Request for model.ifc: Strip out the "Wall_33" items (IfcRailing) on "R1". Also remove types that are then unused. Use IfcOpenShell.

First a look at what the model holds.

```python
import ifcopenshell
import ifcopenshell.util.element

model = ifcopenshell.open("model.ifc")
print(model.schema)
storey = next(s for s in model.by_type("IfcBuildingStorey") if s.Name == "R1")
railings = [e for e in ifcopenshell.util.element.get_decomposition(storey) if e.is_a("IfcRailing")]
seen = {}
for e in railings:
    element_type = ifcopenshell.util.element.get_type(e)
    name = element_type.Name if element_type not in (None, e) else None
    seen[name] = seen.get(name, 0) + 1
for name, count in sorted(seen.items(), key=str):
    print(count, "x", name)
```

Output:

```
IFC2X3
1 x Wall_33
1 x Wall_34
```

```python
import ifcopenshell
import ifcopenshell.api.root
import ifcopenshell.util.element

model = ifcopenshell.open("model.ifc")

storey = next(s for s in model.by_type("IfcBuildingStorey") if s.Name == "R1")
railings = [e for e in ifcopenshell.util.element.get_decomposition(storey) if e.is_a("IfcRailing")]
targets = [e for e in railings if (t := ifcopenshell.util.element.get_type(e)) not in (None, e) and t.Name == "Wall_33"]
types = {ifcopenshell.util.element.get_type(e) for e in targets} - {None, *targets}

for e in targets:
    ifcopenshell.api.root.remove_product(model, product=e)
print(len(targets), "removed")

unused = [t for t in types if not ifcopenshell.util.element.get_types(t)]
for t in unused:
    ifcopenshell.api.root.remove_product(model, product=t)
print(len(unused), "unused types removed")

model.write("model_edited.ifc")
```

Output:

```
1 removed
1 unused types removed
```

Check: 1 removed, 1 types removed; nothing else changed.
